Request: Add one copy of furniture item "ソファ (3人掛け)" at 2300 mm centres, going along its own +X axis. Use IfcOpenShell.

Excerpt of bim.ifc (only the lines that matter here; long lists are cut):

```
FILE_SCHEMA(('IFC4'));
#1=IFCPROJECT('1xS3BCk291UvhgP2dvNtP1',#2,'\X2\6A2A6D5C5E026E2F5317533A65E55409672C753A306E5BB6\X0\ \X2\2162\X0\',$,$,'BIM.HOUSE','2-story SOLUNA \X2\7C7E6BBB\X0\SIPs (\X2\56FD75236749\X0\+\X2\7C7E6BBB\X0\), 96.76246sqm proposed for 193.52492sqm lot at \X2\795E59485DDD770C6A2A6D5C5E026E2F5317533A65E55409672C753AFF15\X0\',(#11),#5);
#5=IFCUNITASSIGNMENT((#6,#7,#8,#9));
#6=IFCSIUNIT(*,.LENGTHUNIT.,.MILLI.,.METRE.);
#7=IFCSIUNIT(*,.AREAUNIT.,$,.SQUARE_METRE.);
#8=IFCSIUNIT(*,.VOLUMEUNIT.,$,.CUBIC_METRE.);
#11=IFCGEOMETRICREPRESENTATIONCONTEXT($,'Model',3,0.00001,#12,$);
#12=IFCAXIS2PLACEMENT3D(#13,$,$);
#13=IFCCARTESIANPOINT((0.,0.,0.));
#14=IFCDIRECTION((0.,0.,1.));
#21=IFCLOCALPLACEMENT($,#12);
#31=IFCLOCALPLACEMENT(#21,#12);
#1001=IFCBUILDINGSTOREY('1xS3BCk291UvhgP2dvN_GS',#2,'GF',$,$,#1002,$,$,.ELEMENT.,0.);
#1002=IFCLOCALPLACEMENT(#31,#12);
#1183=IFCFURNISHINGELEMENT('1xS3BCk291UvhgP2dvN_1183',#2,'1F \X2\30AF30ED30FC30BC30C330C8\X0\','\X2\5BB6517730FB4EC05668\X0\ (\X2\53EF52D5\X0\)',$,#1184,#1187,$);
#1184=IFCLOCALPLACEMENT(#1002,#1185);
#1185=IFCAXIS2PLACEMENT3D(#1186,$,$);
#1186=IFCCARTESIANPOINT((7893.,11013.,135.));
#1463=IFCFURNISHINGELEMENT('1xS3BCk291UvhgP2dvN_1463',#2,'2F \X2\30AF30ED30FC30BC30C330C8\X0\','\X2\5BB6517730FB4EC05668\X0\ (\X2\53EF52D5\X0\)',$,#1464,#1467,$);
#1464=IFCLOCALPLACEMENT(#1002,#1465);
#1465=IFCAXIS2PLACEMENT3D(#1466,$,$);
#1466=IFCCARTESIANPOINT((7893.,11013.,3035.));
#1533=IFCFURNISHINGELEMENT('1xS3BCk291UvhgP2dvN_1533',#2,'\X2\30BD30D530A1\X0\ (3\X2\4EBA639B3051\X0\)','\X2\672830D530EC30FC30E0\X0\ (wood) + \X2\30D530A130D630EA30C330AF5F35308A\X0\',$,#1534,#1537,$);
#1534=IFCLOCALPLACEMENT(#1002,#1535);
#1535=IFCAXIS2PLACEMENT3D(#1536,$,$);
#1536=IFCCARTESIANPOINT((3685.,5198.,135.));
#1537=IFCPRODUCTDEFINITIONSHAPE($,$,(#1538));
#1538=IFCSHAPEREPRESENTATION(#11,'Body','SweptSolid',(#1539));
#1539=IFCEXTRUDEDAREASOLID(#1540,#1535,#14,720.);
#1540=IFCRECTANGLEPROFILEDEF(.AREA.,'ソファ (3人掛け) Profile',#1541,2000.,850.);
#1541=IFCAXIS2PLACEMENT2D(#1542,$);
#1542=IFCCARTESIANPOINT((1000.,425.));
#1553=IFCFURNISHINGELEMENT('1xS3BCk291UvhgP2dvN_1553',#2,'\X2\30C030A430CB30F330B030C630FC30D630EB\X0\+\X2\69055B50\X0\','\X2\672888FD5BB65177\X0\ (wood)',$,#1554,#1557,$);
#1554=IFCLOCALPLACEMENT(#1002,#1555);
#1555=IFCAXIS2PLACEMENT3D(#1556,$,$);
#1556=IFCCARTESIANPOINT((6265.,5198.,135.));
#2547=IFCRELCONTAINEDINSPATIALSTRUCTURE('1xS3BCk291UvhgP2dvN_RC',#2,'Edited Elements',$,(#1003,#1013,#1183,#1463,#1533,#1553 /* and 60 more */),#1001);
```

```python
import ifcopenshell
import ifcopenshell.api.geometry
import ifcopenshell.api.root
import ifcopenshell.util.element
import ifcopenshell.util.placement

model = ifcopenshell.open("bim.ifc")


def reuse_history(source, copy):
    """copy_class also copies each property set's owner history, people and application; keep the originals."""
    for rel in copy.IsDefinedBy:
        if rel.is_a("IfcRelDefinesByProperties") and (history := rel.RelatingPropertyDefinition.OwnerHistory):
            rel.RelatingPropertyDefinition.OwnerHistory = source.OwnerHistory
            ifcopenshell.util.element.remove_deep2(model, history)


source = model.by_guid("1xS3BCk291UvhgP2dvN_1533")
base = ifcopenshell.util.placement.get_local_placement(source.ObjectPlacement)
step = base[:3, 0] * 2300.0

for i in range(1, 2):
    copy = ifcopenshell.api.root.copy_class(model, product=source)
    copy.Representation = ifcopenshell.util.element.copy_deep(
        model, source.Representation, exclude=["IfcGeometricRepresentationContext", "IfcRepresentationMap"]
    )
    reuse_history(source, copy)
    matrix = base.copy()
    matrix[:3, 3] += i * step
    print("added at", matrix[:3, 3].round(3) + 0.0)
    ifcopenshell.api.geometry.edit_object_placement(model, product=copy, matrix=matrix, is_si=False)

model.write("bim_v2.ifc")
```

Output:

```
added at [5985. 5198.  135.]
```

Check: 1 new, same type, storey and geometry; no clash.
